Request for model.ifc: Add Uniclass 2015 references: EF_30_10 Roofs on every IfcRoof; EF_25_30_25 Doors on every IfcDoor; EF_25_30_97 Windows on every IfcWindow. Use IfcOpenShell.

First a look at what the model holds.

```python
import ifcopenshell

model = ifcopenshell.open("model.ifc")
print(model.schema)
print("classifications:", [c.Name for c in model.by_type("IfcClassification")])
for ifc_class in ("IfcDoor", "IfcRoof", "IfcStair", "IfcWall", "IfcWindow"):
    print(ifc_class, len(model.by_type(ifc_class)))
```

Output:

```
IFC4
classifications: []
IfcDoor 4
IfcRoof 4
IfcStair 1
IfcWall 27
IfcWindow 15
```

```python
import ifcopenshell
import ifcopenshell.api.classification

model = ifcopenshell.open("model.ifc")

system = ifcopenshell.api.classification.add_classification(model, classification="Uniclass 2015")

codes = {
    "IfcRoof": ("EF_30_10", "Roofs"),
    "IfcDoor": ("EF_25_30_25", "Doors"),
    "IfcWindow": ("EF_25_30_97", "Windows"),
}
for ifc_class, (code, name) in codes.items():
    products = model.by_type(ifc_class)
    ifcopenshell.api.classification.add_reference(
        model, products=products, classification=system, identification=code, name=name
    )
    print(code, len(products))

model.write("model_edited.ifc")
```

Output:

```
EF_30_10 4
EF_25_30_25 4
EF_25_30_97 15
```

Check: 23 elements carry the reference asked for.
